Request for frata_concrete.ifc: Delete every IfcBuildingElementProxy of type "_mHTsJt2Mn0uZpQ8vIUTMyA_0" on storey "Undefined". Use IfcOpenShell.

First a look at what the model holds.

```python
import ifcopenshell
import ifcopenshell.util.element

model = ifcopenshell.open("frata_concrete.ifc")
print(model.schema)
storey = next(s for s in model.by_type("IfcBuildingStorey") if s.Name == "Undefined")
proxies = [e for e in ifcopenshell.util.element.get_decomposition(storey) if e.is_a("IfcBuildingElementProxy")]
seen = {}
for e in proxies:
    element_type = ifcopenshell.util.element.get_type(e)
    name = element_type.Name if element_type not in (None, e) else None
    seen[name] = seen.get(name, 0) + 1
for name, count in sorted(seen.items(), key=str):
    print(count, "x", name)
```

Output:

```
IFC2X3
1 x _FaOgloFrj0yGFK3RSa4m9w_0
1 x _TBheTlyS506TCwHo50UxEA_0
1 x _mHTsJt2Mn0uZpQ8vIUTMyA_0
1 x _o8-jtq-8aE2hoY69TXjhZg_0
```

```python
import ifcopenshell
import ifcopenshell.api.root
import ifcopenshell.util.element

model = ifcopenshell.open("frata_concrete.ifc")

storey = next(s for s in model.by_type("IfcBuildingStorey") if s.Name == "Undefined")
proxies = [e for e in ifcopenshell.util.element.get_decomposition(storey) if e.is_a("IfcBuildingElementProxy")]
targets = [e for e in proxies if (t := ifcopenshell.util.element.get_type(e)) not in (None, e) and t.Name == "_mHTsJt2Mn0uZpQ8vIUTMyA_0"]

for e in targets:
    ifcopenshell.api.root.remove_product(model, product=e)
print(len(targets), "removed")

model.write("frata_concrete_rev.ifc")
```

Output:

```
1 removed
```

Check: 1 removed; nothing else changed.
